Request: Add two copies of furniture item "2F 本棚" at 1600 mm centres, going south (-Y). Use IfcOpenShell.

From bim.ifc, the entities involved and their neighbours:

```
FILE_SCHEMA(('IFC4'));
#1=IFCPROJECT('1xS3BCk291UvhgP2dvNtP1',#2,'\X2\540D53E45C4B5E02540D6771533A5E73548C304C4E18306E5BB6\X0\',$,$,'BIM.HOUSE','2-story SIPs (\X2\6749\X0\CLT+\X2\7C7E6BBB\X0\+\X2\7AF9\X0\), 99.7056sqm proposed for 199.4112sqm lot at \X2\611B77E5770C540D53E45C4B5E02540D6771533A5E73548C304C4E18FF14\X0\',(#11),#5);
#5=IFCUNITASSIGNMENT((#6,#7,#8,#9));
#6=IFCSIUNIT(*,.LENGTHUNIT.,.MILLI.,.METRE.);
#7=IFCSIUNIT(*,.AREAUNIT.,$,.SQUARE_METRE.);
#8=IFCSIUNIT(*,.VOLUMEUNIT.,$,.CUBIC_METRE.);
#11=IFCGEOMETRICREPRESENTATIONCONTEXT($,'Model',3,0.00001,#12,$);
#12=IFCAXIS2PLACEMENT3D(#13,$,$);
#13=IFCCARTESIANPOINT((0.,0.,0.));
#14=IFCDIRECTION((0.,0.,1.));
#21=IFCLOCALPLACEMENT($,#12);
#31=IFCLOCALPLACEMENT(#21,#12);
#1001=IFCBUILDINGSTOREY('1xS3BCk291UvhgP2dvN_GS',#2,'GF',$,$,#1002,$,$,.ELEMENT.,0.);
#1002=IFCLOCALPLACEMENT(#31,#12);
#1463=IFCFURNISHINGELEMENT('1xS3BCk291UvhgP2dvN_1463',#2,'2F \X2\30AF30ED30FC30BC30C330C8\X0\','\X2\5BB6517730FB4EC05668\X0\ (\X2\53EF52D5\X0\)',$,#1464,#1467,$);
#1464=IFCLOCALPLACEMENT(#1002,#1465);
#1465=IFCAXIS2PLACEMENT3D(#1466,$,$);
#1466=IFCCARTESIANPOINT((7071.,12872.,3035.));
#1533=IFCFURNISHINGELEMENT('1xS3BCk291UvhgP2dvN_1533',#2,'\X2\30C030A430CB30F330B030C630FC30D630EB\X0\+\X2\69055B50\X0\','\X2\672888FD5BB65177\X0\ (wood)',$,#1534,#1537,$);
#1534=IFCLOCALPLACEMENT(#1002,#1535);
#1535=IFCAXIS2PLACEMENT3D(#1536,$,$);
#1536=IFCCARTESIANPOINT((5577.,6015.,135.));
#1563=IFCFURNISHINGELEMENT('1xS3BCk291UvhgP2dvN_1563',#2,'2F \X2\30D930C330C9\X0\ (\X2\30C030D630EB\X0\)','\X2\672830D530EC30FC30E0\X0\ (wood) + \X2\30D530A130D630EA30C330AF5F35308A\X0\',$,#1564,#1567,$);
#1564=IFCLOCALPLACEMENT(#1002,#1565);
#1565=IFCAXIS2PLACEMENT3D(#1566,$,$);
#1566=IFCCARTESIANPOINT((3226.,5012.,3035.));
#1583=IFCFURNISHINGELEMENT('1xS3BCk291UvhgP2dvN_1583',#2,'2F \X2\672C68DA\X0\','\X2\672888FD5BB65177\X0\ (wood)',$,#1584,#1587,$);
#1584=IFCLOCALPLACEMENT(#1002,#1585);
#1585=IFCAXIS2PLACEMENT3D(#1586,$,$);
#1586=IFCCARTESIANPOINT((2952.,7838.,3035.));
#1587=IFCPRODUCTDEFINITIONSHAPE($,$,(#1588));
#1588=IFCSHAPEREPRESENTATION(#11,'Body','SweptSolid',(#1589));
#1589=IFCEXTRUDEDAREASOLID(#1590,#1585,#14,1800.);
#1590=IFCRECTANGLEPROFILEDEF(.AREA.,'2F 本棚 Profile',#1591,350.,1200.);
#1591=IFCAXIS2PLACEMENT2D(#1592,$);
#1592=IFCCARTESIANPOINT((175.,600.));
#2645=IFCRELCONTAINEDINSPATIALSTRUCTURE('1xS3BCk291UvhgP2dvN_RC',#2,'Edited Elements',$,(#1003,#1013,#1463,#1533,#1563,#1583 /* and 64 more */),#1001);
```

```python
import numpy as np
import ifcopenshell
import ifcopenshell.api.geometry
import ifcopenshell.api.root
import ifcopenshell.util.element
import ifcopenshell.util.placement
import ifcopenshell.util.unit

model = ifcopenshell.open("bim.ifc")
unit_scale = ifcopenshell.util.unit.calculate_unit_scale(model)


def reuse_history(source, copy):
    """copy_class also copies each property set's owner history, people and application; keep the originals."""
    for rel in copy.IsDefinedBy:
        if rel.is_a("IfcRelDefinesByProperties") and (history := rel.RelatingPropertyDefinition.OwnerHistory):
            rel.RelatingPropertyDefinition.OwnerHistory = source.OwnerHistory
            ifcopenshell.util.element.remove_deep2(model, history)


source = model.by_id(1583)
base = ifcopenshell.util.placement.get_local_placement(source.ObjectPlacement)
step = np.array([0.0, -1.0, 0.0]) * 1.6 / unit_scale

for i in range(1, 3):
    copy = ifcopenshell.api.root.copy_class(model, product=source)
    copy.Representation = ifcopenshell.util.element.copy_deep(
        model, source.Representation, exclude=["IfcGeometricRepresentationContext", "IfcRepresentationMap"]
    )
    reuse_history(source, copy)
    matrix = base.copy()
    matrix[:3, 3] += i * step
    print("added at", matrix[:3, 3].round(3) + 0.0)
    ifcopenshell.api.geometry.edit_object_placement(model, product=copy, matrix=matrix, is_si=False)

model.write("bim_edited.ifc")
```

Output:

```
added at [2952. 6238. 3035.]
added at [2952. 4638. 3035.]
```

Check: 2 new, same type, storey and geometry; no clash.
